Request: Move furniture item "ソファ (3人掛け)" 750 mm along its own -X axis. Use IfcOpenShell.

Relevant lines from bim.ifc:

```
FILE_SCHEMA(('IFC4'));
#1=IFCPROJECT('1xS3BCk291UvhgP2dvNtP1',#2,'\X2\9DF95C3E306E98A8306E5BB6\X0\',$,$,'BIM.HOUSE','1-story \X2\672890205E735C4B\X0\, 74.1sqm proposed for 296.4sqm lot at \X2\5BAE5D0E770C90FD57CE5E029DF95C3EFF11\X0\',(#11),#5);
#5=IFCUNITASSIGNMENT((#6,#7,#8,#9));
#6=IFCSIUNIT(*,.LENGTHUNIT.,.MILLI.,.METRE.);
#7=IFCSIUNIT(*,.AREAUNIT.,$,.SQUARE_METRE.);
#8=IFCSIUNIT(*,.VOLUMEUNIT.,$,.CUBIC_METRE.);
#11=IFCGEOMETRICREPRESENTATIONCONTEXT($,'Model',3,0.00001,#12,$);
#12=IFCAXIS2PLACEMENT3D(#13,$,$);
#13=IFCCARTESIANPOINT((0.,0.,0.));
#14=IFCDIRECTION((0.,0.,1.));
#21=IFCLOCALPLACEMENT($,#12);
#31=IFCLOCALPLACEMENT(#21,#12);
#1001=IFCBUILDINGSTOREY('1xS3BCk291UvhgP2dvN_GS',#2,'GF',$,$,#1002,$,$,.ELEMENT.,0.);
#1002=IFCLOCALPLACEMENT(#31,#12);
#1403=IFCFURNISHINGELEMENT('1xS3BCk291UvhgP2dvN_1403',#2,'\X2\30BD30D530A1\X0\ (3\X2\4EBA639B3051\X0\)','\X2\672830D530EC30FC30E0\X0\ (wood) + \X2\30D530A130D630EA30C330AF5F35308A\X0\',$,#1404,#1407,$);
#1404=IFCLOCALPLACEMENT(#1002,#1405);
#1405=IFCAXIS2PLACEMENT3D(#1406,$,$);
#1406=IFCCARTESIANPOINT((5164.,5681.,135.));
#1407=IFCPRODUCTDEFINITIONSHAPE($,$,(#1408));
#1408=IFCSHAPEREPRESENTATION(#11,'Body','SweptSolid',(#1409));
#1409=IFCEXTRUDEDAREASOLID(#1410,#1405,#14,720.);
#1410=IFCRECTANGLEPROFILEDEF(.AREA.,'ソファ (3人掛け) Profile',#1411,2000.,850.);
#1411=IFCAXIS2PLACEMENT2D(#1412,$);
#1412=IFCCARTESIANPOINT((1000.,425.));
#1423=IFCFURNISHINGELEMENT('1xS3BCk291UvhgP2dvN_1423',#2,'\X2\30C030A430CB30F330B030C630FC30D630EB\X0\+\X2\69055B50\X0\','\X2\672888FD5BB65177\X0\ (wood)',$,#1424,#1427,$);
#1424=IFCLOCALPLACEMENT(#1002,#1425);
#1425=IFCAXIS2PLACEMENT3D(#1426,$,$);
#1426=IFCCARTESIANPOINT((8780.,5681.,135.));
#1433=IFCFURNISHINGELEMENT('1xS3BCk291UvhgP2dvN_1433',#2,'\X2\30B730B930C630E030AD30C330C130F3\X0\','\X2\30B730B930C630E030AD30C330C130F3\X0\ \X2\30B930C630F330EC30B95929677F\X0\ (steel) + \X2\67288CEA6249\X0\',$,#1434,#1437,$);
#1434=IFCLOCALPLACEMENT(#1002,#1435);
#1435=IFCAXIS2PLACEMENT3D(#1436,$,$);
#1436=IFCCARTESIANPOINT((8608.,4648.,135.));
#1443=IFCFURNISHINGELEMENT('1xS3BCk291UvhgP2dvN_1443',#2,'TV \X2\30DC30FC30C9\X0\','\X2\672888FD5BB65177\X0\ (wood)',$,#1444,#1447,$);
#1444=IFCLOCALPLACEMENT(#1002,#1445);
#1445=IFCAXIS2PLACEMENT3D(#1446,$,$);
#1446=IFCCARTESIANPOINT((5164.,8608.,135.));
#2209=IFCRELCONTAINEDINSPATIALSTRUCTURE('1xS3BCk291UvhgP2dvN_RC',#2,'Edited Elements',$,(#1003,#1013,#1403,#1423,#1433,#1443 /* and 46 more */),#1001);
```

```python
import ifcopenshell
import ifcopenshell.api.geometry
import ifcopenshell.util.placement

model = ifcopenshell.open("bim.ifc")

item = model.by_guid("1xS3BCk291UvhgP2dvN_1403")
matrix = ifcopenshell.util.placement.get_local_placement(item.ObjectPlacement)
matrix[:3, 3] -= matrix[:3, 0] * 750.0
ifcopenshell.api.geometry.edit_object_placement(model, product=item, matrix=matrix, is_si=False)

print(ifcopenshell.util.placement.get_local_placement(item.ObjectPlacement).round(3) + 0.0)

model.write("bim_rev.ifc")
```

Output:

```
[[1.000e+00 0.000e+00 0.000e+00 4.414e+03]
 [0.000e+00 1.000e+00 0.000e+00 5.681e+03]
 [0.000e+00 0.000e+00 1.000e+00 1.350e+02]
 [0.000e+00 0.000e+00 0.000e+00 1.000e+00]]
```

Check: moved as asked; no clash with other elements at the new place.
